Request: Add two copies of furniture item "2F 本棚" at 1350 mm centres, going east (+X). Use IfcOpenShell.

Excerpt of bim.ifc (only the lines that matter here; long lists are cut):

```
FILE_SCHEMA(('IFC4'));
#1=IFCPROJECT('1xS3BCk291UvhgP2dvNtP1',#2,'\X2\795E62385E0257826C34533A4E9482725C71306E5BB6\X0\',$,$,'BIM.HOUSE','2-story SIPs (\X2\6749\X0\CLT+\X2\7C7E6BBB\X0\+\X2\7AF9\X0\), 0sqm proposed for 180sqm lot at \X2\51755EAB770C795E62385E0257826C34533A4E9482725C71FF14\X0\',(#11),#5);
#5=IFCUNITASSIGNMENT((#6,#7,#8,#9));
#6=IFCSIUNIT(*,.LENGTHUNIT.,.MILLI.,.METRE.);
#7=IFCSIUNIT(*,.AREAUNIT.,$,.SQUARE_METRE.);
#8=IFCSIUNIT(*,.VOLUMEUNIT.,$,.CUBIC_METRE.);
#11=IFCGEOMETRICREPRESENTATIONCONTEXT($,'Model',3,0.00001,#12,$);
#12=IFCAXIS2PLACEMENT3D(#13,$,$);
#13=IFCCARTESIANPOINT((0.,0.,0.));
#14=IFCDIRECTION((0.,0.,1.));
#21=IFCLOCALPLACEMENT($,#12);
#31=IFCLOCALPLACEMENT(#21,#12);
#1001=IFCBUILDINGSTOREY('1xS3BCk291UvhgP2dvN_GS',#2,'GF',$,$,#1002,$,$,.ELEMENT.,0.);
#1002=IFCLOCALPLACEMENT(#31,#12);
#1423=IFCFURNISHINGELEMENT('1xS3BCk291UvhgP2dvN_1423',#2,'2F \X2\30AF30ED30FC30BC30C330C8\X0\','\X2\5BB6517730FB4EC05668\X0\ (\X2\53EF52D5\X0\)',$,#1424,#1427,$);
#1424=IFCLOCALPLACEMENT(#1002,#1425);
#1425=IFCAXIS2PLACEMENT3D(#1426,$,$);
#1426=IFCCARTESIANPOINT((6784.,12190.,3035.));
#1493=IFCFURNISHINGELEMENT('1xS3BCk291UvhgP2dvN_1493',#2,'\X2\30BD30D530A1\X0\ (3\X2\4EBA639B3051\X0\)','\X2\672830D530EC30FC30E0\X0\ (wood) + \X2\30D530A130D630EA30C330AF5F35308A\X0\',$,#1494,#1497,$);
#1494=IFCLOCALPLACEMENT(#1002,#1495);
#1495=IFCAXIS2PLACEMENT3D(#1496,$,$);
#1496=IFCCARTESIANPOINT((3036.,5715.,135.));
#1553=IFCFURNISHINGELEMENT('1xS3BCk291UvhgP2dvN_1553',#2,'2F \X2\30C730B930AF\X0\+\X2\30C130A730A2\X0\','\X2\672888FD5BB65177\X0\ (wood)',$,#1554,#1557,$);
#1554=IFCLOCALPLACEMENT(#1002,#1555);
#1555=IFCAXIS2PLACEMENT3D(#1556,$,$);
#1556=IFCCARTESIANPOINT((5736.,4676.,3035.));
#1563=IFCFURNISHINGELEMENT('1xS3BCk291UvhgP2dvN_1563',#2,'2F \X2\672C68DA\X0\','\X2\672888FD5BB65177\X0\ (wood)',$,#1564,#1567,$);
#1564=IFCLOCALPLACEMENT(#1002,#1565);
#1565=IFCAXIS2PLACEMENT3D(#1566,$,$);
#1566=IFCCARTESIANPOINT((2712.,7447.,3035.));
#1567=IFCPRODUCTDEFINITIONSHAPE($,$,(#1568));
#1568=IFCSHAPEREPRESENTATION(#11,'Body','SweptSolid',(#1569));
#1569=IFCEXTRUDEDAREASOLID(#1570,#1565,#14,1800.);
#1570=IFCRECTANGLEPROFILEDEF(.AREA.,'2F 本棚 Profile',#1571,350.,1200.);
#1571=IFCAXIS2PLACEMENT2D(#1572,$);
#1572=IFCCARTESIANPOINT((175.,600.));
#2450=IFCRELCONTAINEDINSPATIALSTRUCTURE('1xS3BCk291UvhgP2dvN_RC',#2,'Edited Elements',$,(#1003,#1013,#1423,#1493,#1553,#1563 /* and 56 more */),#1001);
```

```python
import numpy as np
import ifcopenshell
import ifcopenshell.api.geometry
import ifcopenshell.api.root
import ifcopenshell.util.element
import ifcopenshell.util.placement
import ifcopenshell.util.unit

model = ifcopenshell.open("bim.ifc")
unit_scale = ifcopenshell.util.unit.calculate_unit_scale(model)


def reuse_history(source, copy):
    """copy_class also copies each property set's owner history, people and application; keep the originals."""
    for rel in copy.IsDefinedBy:
        if rel.is_a("IfcRelDefinesByProperties") and (history := rel.RelatingPropertyDefinition.OwnerHistory):
            rel.RelatingPropertyDefinition.OwnerHistory = source.OwnerHistory
            ifcopenshell.util.element.remove_deep2(model, history)


source = model.by_id(1563)
base = ifcopenshell.util.placement.get_local_placement(source.ObjectPlacement)
step = np.array([1.0, 0.0, 0.0]) * 1.35 / unit_scale

for i in range(1, 3):
    copy = ifcopenshell.api.root.copy_class(model, product=source)
    copy.Representation = ifcopenshell.util.element.copy_deep(
        model, source.Representation, exclude=["IfcGeometricRepresentationContext", "IfcRepresentationMap"]
    )
    reuse_history(source, copy)
    matrix = base.copy()
    matrix[:3, 3] += i * step
    print("added at", matrix[:3, 3].round(3) + 0.0)
    ifcopenshell.api.geometry.edit_object_placement(model, product=copy, matrix=matrix, is_si=False)

model.write("bim_edited.ifc")
```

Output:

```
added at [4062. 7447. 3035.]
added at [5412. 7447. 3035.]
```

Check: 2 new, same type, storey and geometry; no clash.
